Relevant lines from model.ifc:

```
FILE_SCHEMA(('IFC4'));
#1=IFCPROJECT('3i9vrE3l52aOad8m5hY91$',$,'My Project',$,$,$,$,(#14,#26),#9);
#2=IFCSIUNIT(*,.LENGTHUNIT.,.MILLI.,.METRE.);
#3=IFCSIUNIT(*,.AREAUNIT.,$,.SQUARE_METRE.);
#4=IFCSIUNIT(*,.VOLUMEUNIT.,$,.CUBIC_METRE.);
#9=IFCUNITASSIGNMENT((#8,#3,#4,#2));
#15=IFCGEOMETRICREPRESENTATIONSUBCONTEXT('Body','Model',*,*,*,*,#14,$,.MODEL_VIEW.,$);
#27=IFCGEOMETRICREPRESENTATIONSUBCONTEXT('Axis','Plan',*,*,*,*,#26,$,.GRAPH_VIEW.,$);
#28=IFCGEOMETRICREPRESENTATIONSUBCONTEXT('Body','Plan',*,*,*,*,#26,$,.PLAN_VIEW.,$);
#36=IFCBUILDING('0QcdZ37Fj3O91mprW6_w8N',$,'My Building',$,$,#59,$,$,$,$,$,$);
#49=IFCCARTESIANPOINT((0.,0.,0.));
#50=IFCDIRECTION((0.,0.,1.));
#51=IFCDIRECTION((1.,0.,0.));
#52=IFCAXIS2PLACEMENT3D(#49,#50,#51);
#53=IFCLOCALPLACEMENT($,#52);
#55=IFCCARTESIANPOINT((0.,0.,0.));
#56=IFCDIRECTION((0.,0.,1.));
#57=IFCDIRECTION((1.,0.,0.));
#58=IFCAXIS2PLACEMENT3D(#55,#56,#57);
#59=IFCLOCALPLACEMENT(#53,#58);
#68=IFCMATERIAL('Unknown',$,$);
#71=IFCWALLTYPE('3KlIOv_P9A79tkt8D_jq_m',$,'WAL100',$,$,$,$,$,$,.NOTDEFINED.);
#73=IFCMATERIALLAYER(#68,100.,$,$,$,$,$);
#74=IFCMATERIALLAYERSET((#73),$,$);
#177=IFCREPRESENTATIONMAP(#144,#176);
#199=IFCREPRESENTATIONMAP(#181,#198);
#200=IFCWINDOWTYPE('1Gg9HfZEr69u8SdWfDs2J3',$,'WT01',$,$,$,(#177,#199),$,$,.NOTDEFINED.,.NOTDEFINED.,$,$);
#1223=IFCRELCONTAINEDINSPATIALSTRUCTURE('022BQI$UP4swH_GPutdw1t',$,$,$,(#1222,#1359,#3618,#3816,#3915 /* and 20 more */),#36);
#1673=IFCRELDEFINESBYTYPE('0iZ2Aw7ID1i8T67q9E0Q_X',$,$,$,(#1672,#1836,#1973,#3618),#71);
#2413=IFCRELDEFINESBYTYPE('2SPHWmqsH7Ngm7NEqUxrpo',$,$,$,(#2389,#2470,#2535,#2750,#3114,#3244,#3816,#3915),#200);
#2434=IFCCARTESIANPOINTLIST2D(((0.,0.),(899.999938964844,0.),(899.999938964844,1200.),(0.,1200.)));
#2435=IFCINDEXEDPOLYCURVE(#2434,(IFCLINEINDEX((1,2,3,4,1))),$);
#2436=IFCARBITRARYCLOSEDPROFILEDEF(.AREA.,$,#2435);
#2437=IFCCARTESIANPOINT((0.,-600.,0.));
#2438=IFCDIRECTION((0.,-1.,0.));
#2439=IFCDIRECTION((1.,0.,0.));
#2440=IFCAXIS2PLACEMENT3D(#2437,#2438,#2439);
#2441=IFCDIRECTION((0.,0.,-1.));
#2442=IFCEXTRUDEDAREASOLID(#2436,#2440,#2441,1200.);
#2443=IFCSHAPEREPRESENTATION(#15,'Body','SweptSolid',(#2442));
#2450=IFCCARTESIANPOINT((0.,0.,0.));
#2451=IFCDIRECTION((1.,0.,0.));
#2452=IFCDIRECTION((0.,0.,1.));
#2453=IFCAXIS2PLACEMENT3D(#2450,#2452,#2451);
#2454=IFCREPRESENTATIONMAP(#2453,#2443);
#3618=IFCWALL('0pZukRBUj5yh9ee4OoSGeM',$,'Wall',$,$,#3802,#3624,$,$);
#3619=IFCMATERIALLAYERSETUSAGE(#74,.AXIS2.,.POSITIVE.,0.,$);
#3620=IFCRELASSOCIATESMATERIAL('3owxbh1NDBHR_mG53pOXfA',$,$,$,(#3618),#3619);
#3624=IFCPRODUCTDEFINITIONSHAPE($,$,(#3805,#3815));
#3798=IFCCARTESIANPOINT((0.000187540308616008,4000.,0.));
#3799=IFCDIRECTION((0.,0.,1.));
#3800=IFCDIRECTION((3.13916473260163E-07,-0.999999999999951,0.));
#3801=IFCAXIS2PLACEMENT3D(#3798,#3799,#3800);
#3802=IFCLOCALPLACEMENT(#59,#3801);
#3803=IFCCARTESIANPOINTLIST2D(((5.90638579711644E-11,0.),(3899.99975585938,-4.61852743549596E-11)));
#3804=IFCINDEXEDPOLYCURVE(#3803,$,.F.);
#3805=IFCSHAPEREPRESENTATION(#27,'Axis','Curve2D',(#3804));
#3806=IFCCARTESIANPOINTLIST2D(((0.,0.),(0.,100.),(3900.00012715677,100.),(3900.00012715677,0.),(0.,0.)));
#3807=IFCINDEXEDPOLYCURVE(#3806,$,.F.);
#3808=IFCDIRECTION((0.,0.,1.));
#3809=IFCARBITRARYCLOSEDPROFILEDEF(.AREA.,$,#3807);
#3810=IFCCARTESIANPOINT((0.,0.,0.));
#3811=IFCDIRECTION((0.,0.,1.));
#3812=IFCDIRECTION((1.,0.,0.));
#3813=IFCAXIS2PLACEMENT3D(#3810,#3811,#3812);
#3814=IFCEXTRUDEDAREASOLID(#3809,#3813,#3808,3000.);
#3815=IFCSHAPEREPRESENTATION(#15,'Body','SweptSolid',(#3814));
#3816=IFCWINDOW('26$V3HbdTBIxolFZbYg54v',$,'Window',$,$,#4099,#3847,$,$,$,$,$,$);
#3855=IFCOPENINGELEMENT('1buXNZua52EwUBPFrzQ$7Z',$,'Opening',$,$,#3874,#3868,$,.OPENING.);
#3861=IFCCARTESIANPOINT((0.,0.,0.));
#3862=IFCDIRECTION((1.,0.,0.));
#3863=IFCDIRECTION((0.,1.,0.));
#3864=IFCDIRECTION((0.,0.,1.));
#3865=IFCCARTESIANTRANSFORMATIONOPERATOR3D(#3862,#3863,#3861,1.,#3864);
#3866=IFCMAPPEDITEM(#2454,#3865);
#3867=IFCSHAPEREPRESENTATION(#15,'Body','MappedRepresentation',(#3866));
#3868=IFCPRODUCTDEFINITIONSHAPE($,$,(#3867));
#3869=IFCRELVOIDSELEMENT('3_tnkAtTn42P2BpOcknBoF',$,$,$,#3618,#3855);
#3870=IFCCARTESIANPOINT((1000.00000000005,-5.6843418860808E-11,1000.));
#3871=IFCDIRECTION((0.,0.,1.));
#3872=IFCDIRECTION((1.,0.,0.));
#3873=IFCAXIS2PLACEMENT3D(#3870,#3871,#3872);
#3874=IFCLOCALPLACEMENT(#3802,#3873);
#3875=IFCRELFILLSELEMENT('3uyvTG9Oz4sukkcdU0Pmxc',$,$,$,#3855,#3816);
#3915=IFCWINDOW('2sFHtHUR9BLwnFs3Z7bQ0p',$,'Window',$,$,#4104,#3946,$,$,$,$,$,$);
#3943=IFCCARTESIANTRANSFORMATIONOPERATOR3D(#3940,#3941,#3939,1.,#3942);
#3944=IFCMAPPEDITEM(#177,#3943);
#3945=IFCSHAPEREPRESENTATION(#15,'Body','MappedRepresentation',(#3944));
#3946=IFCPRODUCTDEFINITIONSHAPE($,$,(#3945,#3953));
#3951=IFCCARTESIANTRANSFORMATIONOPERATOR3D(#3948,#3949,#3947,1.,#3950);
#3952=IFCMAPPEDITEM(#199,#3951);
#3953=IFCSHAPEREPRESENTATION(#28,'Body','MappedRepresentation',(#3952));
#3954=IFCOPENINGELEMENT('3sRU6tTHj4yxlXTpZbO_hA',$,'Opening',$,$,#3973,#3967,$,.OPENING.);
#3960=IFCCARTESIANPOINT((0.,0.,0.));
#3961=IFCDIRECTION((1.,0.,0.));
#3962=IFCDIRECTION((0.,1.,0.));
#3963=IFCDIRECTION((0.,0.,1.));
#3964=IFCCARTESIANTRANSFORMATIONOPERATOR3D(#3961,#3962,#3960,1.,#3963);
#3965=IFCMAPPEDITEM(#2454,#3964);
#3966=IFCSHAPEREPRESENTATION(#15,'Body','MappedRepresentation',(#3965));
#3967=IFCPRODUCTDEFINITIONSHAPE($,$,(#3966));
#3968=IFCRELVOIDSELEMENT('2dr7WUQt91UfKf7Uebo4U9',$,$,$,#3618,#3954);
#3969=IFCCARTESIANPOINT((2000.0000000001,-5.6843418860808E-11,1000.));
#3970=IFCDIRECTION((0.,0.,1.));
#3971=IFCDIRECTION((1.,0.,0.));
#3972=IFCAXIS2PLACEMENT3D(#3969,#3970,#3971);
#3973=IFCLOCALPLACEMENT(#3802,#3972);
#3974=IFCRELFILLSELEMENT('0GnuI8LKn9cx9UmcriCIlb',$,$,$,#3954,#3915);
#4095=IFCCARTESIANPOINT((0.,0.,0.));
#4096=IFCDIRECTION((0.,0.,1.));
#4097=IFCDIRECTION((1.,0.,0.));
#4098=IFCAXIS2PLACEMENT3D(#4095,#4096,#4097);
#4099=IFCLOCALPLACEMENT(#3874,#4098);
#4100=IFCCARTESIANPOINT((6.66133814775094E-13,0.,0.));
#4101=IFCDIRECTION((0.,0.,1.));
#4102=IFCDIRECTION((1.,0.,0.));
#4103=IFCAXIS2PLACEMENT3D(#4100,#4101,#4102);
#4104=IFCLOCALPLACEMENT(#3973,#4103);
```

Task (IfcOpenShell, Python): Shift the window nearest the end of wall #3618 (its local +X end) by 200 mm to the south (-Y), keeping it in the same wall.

```python
import ifcopenshell
import ifcopenshell.api.geometry
import ifcopenshell.util.placement
import ifcopenshell.util.unit

model = ifcopenshell.open("model.ifc")
unit_scale = ifcopenshell.util.unit.calculate_unit_scale(model)

window = model.by_id(3915)
opening = window.FillsVoids[0].RelatingOpeningElement
wall = opening.VoidsElements[0].RelatingBuildingElement

wall_matrix = ifcopenshell.util.placement.get_local_placement(wall.ObjectPlacement)
shift = wall_matrix[:3, 0] * 0.2 / unit_scale
before = ifcopenshell.util.placement.get_local_placement(window.ObjectPlacement)[:3, 3].copy()

# The window is placed relative to its opening, so it follows when the opening moves.
matrix = ifcopenshell.util.placement.get_local_placement(opening.ObjectPlacement)
matrix[:3, 3] += shift
ifcopenshell.api.geometry.edit_object_placement(
    model, product=opening, matrix=matrix, is_si=False, should_transform_children=True
)

after = ifcopenshell.util.placement.get_local_placement(window.ObjectPlacement)[:3, 3]
print("window moved by", (after - before).round(3) + 0.0)

model.write("model_v2.ifc")
```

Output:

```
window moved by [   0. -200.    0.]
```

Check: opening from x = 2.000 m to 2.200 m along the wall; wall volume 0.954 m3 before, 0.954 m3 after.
